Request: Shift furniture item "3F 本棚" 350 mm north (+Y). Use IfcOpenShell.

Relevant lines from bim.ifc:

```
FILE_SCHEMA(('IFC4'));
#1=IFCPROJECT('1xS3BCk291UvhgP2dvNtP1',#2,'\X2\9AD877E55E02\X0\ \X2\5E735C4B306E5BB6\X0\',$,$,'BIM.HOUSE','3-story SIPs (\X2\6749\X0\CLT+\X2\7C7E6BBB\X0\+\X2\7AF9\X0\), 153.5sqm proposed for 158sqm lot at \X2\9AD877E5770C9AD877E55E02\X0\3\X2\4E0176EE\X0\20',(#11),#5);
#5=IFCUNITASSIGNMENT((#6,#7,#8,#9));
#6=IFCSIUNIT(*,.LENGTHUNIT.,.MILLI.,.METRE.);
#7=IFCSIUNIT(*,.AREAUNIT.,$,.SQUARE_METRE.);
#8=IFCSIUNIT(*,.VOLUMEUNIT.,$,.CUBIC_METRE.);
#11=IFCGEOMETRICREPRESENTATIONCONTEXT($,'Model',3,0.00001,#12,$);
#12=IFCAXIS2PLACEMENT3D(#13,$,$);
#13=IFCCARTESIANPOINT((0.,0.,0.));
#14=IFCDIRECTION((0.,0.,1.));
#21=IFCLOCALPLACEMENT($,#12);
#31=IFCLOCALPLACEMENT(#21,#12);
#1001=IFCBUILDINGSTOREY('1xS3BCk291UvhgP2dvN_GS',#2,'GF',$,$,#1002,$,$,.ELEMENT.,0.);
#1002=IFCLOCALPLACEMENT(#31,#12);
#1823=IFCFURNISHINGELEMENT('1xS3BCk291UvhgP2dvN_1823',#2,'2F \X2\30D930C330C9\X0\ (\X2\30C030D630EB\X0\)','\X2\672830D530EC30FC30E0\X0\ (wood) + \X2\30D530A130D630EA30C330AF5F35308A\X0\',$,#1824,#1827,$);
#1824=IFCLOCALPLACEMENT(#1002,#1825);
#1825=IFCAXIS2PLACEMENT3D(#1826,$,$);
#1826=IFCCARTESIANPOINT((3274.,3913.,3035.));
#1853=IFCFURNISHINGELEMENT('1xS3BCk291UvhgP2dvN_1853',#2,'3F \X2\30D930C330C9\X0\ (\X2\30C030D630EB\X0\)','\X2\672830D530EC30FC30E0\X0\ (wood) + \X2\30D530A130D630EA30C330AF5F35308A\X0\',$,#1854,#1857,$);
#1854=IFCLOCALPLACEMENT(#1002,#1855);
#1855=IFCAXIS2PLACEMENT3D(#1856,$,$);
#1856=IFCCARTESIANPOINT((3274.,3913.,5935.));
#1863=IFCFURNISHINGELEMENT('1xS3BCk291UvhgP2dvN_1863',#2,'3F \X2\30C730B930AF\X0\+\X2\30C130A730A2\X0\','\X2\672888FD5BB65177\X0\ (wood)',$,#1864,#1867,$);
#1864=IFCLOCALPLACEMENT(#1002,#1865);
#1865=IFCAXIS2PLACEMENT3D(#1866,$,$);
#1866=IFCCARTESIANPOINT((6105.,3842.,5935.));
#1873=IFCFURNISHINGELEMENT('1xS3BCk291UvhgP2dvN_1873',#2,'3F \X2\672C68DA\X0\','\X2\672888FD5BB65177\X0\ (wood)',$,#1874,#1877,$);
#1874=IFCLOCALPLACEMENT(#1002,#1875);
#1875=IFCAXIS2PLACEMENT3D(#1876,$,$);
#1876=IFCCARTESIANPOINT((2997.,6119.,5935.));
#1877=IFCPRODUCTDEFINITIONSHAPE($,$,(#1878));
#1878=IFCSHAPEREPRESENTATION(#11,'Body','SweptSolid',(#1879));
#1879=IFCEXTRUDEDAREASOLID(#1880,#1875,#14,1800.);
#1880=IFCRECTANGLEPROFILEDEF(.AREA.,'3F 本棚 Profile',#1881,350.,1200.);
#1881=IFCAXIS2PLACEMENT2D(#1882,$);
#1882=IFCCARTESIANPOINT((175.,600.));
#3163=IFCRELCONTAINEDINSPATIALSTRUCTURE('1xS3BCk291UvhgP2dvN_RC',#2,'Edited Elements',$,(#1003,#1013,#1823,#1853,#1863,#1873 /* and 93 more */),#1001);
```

```python
import ifcopenshell
import ifcopenshell.api.geometry
import ifcopenshell.util.placement

model = ifcopenshell.open("bim.ifc")

item = model.by_guid("1xS3BCk291UvhgP2dvN_1873")
matrix = ifcopenshell.util.placement.get_local_placement(item.ObjectPlacement)
matrix[1, 3] += 350.0
ifcopenshell.api.geometry.edit_object_placement(model, product=item, matrix=matrix, is_si=False)

print(ifcopenshell.util.placement.get_local_placement(item.ObjectPlacement).round(3) + 0.0)

model.write("bim-out.ifc")
```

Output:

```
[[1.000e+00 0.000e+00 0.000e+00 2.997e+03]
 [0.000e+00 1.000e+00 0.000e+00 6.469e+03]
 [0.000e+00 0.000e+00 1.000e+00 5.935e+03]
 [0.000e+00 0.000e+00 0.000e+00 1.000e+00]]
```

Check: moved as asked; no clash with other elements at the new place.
